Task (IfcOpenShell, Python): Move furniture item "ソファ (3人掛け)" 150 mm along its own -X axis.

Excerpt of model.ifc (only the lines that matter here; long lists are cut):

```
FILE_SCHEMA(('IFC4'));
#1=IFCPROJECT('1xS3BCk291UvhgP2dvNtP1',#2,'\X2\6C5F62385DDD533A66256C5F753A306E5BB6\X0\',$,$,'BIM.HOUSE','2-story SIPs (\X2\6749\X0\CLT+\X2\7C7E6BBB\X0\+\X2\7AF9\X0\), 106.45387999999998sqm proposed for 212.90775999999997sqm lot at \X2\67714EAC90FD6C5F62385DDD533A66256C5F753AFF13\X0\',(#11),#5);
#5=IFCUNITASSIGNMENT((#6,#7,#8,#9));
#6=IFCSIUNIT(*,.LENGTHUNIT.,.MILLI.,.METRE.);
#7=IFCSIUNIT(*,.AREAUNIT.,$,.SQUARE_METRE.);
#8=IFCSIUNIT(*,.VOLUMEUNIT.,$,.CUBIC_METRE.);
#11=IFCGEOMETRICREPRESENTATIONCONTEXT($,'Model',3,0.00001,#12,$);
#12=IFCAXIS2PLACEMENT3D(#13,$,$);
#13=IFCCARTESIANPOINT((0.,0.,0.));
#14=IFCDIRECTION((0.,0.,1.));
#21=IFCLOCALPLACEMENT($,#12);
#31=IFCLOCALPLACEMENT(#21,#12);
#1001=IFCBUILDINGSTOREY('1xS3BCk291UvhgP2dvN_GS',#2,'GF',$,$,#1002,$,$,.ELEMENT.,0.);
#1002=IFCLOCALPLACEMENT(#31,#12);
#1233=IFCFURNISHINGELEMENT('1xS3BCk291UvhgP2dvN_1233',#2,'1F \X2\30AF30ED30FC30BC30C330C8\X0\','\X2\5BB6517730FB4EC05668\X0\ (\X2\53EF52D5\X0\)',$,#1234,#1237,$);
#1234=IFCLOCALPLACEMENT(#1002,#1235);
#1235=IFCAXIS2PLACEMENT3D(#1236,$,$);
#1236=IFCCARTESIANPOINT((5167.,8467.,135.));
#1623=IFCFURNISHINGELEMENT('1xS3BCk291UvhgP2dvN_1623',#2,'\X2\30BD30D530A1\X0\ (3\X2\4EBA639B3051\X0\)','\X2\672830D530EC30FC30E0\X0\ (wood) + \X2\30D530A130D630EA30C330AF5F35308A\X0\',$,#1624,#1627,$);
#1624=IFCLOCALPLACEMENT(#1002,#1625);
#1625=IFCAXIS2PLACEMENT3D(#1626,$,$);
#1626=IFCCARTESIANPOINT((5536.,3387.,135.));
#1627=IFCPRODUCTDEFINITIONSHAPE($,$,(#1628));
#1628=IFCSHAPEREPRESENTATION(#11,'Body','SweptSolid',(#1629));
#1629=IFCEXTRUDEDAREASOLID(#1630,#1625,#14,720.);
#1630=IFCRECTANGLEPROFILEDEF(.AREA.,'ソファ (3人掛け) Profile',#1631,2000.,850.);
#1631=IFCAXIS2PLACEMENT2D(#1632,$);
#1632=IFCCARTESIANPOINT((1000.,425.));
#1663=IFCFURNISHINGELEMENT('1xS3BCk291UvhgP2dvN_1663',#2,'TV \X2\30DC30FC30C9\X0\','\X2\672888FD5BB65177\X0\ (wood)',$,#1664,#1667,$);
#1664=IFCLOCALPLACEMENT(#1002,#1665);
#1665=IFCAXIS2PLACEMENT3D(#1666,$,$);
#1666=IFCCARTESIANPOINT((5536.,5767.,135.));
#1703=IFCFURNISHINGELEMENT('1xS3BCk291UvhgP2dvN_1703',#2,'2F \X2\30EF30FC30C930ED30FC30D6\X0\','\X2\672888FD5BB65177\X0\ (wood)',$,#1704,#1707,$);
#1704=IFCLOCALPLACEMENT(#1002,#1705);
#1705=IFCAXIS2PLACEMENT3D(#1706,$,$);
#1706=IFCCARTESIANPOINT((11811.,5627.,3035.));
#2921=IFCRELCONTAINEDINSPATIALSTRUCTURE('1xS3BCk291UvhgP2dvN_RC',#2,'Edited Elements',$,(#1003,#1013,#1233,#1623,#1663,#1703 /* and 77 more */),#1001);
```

```python
import ifcopenshell
import ifcopenshell.api.geometry
import ifcopenshell.util.placement

model = ifcopenshell.open("model.ifc")

item = model.by_id(1623)
matrix = ifcopenshell.util.placement.get_local_placement(item.ObjectPlacement)
matrix[:3, 3] -= matrix[:3, 0] * 150.0
ifcopenshell.api.geometry.edit_object_placement(model, product=item, matrix=matrix, is_si=False)

print(ifcopenshell.util.placement.get_local_placement(item.ObjectPlacement).round(3) + 0.0)

model.write("model_updated.ifc")
```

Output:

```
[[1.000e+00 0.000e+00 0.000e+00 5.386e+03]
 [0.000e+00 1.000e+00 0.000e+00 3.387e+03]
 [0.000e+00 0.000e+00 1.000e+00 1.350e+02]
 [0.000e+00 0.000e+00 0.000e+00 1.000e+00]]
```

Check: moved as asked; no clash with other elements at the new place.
